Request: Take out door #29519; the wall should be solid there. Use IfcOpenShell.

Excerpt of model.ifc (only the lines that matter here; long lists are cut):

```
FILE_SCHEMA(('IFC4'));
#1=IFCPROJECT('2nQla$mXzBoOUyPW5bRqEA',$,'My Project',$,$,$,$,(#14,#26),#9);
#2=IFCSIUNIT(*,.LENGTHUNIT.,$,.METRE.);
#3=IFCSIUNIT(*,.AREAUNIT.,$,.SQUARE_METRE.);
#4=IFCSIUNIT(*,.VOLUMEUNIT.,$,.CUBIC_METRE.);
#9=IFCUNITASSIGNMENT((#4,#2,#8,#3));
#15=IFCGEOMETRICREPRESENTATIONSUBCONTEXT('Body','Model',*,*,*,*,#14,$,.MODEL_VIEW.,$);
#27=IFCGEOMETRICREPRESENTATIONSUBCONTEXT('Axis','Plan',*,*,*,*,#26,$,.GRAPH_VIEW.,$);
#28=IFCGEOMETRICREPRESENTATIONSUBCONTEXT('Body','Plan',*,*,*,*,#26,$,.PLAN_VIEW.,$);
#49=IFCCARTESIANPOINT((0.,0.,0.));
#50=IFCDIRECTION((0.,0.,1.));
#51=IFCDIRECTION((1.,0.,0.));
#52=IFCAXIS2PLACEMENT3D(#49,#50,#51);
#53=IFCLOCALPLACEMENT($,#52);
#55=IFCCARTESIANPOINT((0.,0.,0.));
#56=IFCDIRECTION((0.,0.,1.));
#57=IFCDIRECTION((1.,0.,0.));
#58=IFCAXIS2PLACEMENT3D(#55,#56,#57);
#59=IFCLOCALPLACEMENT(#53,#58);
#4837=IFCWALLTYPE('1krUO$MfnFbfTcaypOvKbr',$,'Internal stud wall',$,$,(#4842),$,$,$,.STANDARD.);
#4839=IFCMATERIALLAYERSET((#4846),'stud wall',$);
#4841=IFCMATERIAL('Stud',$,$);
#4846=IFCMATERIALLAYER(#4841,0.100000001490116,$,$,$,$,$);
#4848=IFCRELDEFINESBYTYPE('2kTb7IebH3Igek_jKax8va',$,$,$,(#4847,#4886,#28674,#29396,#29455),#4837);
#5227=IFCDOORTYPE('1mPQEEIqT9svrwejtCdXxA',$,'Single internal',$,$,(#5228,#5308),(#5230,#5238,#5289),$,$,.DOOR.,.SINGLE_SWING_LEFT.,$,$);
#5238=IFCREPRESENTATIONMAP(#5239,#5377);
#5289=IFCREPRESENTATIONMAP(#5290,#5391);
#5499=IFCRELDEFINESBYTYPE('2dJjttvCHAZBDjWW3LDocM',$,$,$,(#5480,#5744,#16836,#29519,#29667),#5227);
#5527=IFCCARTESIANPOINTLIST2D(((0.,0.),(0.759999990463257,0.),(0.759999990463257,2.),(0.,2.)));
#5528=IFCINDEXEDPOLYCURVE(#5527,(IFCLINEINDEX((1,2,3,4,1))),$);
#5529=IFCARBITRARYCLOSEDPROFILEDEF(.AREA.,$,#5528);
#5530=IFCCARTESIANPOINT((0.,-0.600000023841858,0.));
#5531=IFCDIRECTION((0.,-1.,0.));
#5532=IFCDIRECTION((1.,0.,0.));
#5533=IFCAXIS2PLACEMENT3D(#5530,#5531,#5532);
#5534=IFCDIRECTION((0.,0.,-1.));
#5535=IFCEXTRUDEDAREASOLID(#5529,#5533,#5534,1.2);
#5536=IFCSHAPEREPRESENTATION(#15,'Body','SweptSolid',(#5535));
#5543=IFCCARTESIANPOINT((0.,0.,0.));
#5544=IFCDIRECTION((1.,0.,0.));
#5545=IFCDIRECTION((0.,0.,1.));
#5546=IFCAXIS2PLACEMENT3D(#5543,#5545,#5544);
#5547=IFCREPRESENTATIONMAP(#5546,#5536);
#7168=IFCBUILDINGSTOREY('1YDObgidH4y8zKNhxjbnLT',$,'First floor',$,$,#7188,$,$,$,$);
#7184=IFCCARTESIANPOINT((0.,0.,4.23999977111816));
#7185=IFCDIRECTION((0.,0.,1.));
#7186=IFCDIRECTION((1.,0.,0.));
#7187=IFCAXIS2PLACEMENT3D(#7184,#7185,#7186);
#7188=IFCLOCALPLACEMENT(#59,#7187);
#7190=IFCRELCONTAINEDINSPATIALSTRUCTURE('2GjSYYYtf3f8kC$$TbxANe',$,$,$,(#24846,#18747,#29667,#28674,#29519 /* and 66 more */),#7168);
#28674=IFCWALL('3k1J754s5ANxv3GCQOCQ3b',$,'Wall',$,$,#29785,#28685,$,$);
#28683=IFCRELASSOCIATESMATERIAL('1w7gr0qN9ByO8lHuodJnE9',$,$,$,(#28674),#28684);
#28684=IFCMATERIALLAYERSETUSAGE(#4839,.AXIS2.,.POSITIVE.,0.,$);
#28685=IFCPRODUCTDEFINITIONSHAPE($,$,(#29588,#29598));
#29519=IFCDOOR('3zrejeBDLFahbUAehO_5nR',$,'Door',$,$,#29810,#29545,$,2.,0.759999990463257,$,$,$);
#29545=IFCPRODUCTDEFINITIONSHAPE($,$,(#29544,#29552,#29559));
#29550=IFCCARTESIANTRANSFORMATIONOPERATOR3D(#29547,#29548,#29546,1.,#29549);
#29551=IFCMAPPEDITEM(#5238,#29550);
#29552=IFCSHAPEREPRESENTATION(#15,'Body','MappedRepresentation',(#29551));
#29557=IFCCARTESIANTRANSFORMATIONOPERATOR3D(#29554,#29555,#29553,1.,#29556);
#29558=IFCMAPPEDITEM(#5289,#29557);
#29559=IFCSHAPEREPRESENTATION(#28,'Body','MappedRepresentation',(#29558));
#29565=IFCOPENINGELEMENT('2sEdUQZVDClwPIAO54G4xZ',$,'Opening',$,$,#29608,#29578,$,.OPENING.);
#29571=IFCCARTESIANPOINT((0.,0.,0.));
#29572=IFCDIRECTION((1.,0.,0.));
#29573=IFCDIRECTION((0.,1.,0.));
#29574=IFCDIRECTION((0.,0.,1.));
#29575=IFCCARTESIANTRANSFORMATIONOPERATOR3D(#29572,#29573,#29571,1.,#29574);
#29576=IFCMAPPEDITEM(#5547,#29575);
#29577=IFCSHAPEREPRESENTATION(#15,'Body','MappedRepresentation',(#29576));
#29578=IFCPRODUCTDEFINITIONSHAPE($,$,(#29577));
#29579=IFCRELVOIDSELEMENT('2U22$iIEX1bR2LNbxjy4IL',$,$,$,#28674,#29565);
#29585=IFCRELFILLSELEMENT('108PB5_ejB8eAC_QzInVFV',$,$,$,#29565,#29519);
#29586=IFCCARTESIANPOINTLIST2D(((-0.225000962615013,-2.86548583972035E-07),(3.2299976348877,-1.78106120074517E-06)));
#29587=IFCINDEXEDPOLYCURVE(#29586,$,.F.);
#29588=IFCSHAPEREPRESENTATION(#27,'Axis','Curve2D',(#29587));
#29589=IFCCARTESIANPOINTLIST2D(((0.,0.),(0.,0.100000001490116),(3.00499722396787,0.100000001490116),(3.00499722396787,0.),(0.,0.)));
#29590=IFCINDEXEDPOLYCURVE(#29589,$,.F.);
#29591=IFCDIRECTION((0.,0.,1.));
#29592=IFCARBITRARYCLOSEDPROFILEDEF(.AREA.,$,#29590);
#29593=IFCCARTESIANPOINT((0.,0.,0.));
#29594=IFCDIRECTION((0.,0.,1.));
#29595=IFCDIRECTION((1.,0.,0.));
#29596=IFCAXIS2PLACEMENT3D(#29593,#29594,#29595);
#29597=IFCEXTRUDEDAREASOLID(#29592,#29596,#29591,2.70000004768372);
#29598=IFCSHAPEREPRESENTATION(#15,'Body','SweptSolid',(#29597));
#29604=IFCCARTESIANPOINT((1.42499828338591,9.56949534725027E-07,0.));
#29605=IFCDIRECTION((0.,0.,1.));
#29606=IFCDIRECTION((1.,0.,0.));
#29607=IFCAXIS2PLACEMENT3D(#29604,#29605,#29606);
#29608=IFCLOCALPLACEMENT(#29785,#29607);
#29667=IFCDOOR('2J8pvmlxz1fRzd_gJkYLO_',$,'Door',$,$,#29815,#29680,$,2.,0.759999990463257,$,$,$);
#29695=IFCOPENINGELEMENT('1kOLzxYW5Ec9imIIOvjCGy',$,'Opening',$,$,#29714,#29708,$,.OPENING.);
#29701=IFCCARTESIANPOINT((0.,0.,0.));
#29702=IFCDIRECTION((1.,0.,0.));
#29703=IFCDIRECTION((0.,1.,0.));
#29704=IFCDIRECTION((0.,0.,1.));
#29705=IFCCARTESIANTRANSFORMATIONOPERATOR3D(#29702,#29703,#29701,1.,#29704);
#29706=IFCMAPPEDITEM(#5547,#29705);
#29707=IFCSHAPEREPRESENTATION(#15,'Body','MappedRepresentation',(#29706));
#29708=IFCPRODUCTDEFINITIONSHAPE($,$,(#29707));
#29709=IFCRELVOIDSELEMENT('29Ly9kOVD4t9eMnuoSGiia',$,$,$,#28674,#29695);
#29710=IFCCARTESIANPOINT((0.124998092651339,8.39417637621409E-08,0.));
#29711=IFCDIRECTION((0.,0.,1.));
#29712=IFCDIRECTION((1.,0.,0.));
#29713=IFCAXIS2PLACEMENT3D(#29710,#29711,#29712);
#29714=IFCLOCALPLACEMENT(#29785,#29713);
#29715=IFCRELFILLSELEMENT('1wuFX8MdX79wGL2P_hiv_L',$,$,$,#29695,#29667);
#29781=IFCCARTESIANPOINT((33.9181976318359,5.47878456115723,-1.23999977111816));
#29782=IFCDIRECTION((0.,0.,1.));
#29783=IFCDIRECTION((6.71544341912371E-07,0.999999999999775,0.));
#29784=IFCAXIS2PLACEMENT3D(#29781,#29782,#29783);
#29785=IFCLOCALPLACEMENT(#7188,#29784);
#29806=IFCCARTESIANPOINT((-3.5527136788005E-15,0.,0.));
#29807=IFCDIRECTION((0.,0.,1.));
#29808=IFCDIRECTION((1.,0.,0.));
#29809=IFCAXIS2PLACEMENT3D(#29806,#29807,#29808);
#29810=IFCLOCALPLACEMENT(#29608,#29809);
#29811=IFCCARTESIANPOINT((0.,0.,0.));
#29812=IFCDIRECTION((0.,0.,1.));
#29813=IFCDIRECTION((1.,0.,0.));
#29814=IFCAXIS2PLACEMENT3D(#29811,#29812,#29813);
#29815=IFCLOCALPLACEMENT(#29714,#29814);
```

```python
import ifcopenshell
import ifcopenshell.api.feature
import ifcopenshell.api.root
import ifcopenshell.geom
import ifcopenshell.util.shape

model = ifcopenshell.open("model.ifc")
settings = ifcopenshell.geom.settings()


def volume(element):
    """Net volume in cubic metres, openings subtracted."""
    shape = ifcopenshell.geom.create_shape(settings, element)
    return ifcopenshell.util.shape.get_volume(shape.geometry)


door = model.by_id(29519)
opening = door.FillsVoids[0].RelatingOpeningElement
wall = opening.VoidsElements[0].RelatingBuildingElement
before = volume(wall)

ifcopenshell.api.root.remove_product(model, product=door)
ifcopenshell.api.feature.remove_feature(model, feature=opening)

after = volume(wall)

print(f"wall volume {before:.3f} -> {after:.3f} m3")

model.write("model_edited.ifc")
```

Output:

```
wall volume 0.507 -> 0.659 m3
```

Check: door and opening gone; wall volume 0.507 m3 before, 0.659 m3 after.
